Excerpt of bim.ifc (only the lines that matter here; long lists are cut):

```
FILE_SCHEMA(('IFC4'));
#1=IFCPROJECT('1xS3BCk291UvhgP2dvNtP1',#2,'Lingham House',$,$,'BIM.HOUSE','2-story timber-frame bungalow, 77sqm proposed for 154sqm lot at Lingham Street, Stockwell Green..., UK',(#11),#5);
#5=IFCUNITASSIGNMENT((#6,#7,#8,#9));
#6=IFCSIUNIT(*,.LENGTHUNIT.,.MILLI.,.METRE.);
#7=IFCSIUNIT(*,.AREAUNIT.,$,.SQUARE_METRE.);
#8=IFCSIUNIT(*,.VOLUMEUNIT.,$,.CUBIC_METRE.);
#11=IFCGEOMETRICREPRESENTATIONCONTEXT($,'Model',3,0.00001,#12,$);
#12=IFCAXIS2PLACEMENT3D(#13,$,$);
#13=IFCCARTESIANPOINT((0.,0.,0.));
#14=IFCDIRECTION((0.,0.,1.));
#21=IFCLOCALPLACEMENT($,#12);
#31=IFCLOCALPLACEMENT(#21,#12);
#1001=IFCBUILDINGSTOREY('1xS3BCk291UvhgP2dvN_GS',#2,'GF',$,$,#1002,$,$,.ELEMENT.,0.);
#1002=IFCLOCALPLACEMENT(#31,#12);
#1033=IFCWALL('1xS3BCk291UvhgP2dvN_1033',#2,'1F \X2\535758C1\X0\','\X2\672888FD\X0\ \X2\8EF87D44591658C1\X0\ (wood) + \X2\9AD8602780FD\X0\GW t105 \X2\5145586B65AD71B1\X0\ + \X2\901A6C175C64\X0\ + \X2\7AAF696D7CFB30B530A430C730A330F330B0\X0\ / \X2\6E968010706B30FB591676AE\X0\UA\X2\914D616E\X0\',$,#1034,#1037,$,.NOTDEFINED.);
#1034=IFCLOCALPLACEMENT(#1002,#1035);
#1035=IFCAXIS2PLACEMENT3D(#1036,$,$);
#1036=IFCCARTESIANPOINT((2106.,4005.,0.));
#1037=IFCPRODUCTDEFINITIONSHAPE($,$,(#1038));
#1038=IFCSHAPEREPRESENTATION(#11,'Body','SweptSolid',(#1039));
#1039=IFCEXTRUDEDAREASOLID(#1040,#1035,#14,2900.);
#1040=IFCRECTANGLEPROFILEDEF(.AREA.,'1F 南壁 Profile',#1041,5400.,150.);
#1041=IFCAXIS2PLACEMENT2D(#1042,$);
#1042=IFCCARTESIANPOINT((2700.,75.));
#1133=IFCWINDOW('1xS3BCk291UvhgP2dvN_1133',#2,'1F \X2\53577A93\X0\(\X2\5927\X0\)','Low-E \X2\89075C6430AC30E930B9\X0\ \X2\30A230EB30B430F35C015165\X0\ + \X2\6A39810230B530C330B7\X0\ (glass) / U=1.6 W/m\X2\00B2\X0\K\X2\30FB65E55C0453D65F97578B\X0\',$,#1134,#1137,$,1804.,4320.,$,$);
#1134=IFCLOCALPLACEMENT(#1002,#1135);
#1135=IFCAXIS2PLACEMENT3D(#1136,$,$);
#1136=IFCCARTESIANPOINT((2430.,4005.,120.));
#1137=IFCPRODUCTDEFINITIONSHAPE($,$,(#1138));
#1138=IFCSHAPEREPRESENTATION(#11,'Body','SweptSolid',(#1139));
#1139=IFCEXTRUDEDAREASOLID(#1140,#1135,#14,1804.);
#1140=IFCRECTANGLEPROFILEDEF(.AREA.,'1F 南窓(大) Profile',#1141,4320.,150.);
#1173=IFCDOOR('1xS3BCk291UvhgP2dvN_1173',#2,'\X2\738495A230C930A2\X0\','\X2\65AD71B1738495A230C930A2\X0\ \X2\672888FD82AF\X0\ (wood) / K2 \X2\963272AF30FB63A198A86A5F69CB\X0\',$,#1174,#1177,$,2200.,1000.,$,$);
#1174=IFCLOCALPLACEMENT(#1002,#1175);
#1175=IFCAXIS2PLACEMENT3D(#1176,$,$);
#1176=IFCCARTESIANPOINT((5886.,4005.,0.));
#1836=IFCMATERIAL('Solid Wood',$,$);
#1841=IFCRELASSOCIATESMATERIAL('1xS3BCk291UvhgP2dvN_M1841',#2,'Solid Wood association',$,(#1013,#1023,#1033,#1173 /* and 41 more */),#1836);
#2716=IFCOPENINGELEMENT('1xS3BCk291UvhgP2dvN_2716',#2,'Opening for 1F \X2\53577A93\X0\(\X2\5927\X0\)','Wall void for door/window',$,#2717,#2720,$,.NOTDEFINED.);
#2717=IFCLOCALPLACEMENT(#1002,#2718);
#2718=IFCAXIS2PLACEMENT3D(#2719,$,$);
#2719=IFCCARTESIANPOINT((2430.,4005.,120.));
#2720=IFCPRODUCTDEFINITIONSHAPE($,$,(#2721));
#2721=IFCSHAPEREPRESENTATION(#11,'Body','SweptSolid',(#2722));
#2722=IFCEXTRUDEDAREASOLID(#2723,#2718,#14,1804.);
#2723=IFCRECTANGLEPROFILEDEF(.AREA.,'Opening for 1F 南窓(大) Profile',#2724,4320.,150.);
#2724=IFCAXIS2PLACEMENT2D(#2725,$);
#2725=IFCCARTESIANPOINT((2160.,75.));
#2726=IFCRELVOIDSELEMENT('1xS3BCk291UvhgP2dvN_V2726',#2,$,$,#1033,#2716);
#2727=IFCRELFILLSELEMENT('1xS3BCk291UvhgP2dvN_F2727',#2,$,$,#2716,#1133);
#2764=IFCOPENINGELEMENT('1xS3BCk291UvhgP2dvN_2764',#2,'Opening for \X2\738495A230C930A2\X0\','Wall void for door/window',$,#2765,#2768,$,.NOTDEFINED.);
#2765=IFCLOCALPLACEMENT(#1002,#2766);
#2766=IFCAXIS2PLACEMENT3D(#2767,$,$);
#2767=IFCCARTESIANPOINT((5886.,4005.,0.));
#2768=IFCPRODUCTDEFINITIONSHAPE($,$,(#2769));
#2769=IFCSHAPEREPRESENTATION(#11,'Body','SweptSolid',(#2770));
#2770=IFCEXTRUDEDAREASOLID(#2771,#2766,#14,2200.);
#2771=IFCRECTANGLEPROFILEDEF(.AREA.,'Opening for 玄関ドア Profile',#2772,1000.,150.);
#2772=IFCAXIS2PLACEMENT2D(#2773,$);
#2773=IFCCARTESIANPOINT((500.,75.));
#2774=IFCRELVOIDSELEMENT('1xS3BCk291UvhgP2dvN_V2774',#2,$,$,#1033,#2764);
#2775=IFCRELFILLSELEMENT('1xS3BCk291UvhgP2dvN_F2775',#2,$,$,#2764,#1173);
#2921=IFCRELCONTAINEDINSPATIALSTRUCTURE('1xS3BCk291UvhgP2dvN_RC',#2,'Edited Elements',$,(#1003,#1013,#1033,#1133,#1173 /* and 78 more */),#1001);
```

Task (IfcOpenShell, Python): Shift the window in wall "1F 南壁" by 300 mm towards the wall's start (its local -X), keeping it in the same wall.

```python
import ifcopenshell
import ifcopenshell.api.geometry
import ifcopenshell.util.placement

model = ifcopenshell.open("bim.ifc")

window = model.by_id(1133)
opening = window.FillsVoids[0].RelatingOpeningElement
wall = opening.VoidsElements[0].RelatingBuildingElement

wall_matrix = ifcopenshell.util.placement.get_local_placement(wall.ObjectPlacement)
shift = wall_matrix[:3, 0] * -300.0
before = ifcopenshell.util.placement.get_local_placement(window.ObjectPlacement)[:3, 3].copy()

# The window is not placed relative to its opening, so move both.
for product in (opening, window):
    matrix = ifcopenshell.util.placement.get_local_placement(product.ObjectPlacement)
    matrix[:3, 3] += shift
    ifcopenshell.api.geometry.edit_object_placement(model, product=product, matrix=matrix, is_si=False)

after = ifcopenshell.util.placement.get_local_placement(window.ObjectPlacement)[:3, 3]
print("window moved by", (after - before).round(3) + 0.0)

model.write("bim_v2.ifc")
```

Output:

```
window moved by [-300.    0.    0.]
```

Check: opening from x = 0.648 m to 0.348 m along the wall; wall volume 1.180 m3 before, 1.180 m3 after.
